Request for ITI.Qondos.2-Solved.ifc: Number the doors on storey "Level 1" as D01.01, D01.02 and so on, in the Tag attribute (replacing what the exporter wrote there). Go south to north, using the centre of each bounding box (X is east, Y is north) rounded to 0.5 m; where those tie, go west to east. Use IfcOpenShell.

First a look at what the model holds.

```python
import ifcopenshell
import ifcopenshell.util.element
import ifcopenshell.util.placement

model = ifcopenshell.open("ITI.Qondos.2-Solved.ifc")
print(model.schema)
storey = next(s for s in model.by_type("IfcBuildingStorey") if s.Name == "Level 1")
doors = [e for e in ifcopenshell.util.element.get_decomposition(storey) if e.is_a("IfcDoor")]
for e in sorted(doors, key=lambda e: e.id()):
    origin = ifcopenshell.util.placement.get_local_placement(e.ObjectPlacement)[:3, 3]
    print(e.id(), e.Tag, e.Name, origin.round(2) + 0.0, sep=" | ")
```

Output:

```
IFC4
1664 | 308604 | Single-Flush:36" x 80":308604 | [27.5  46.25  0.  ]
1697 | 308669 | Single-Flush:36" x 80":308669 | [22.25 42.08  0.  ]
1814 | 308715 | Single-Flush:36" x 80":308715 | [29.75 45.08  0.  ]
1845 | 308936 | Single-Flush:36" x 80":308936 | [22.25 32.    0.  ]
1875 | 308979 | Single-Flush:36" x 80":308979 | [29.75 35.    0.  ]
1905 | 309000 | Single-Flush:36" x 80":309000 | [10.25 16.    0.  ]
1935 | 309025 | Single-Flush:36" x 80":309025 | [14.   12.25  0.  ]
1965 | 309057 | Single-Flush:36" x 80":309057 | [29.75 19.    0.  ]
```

```python
import ifcopenshell
import ifcopenshell.geom
import ifcopenshell.util.element
import ifcopenshell.util.shape

model = ifcopenshell.open("ITI.Qondos.2-Solved.ifc")
settings = ifcopenshell.geom.settings()
settings.set("use-world-coords", True)


def centre(element):
    shape = ifcopenshell.geom.create_shape(settings, element)
    return ifcopenshell.util.shape.get_bbox_centroid(shape.geometry)


storey = next(s for s in model.by_type("IfcBuildingStorey") if s.Name == "Level 1")
doors = [e for e in ifcopenshell.util.element.get_decomposition(storey) if e.is_a("IfcDoor")]

# Insertion points can sit at a corner or the storey origin, so sort by the geometry (in metres).
centres = {e: centre(e) for e in doors}
doors.sort(key=lambda e: (round(centres[e][1] / 0.5), centres[e][0]))

for i, e in enumerate(doors, start=1):
    number = f"D01.{i:02d}"
    e.Tag = number
    print(e.id(), number)

model.write("ITI.Qondos.2-Solved_rev.ifc")
```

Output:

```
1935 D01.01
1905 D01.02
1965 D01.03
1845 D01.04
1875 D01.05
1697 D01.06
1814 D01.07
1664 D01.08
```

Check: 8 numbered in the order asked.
